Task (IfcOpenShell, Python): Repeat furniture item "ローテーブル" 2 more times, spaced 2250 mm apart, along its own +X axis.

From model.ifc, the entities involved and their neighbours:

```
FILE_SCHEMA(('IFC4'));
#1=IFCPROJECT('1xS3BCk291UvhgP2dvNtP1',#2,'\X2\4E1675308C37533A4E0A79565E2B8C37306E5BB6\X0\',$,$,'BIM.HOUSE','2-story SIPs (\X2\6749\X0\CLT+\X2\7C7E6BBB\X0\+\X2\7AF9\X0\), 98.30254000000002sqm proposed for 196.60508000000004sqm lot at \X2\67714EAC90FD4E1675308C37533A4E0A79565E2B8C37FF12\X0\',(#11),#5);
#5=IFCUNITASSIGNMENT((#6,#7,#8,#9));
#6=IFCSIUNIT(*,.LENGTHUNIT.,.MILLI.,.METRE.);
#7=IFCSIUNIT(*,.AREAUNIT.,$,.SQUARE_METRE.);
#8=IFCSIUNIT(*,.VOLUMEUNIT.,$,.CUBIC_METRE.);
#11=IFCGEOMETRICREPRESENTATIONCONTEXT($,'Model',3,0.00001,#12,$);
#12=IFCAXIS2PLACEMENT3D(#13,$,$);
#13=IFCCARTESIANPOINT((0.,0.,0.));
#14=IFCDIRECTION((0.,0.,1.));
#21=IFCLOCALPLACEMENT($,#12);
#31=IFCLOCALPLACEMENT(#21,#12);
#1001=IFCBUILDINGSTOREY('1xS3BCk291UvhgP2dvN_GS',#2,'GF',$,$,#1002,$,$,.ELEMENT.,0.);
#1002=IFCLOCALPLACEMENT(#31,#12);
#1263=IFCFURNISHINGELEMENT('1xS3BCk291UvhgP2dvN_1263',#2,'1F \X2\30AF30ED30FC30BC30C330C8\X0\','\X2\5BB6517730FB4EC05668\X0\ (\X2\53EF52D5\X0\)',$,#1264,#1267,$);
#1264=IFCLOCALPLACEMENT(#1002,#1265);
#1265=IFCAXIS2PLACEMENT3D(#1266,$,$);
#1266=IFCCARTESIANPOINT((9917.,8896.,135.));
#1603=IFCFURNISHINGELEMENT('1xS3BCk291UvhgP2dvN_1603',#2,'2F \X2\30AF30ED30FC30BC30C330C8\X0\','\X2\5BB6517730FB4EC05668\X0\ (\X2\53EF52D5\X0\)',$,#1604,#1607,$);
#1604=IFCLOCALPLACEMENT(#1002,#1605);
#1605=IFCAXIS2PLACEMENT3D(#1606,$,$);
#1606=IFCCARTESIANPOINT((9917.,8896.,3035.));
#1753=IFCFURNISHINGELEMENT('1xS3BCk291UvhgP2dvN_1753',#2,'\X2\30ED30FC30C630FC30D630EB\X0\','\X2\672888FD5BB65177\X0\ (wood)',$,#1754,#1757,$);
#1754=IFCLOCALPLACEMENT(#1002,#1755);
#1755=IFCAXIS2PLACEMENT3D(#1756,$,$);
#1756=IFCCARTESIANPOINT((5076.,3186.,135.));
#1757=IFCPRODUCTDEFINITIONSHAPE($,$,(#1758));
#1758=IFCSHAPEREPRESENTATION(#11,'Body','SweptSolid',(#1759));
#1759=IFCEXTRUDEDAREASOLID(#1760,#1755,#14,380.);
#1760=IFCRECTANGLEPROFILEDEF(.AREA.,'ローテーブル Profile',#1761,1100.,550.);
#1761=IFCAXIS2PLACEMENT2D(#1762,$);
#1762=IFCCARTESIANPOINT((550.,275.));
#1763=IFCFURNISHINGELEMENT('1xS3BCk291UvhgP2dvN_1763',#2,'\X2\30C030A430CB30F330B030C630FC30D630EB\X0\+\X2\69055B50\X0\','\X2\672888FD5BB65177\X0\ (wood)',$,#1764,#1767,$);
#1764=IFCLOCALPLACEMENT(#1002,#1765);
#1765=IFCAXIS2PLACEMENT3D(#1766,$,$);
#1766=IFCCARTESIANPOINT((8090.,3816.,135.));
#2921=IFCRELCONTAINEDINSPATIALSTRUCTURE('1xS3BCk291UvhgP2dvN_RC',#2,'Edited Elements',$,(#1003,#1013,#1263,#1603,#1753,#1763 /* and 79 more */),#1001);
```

```python
import ifcopenshell
import ifcopenshell.api.geometry
import ifcopenshell.api.root
import ifcopenshell.util.element
import ifcopenshell.util.placement
import ifcopenshell.util.unit

model = ifcopenshell.open("model.ifc")
unit_scale = ifcopenshell.util.unit.calculate_unit_scale(model)


def reuse_history(source, copy):
    """copy_class also copies each property set's owner history, people and application; keep the originals."""
    for rel in copy.IsDefinedBy:
        if rel.is_a("IfcRelDefinesByProperties") and (history := rel.RelatingPropertyDefinition.OwnerHistory):
            rel.RelatingPropertyDefinition.OwnerHistory = source.OwnerHistory
            ifcopenshell.util.element.remove_deep2(model, history)


source = model.by_id(1753)
base = ifcopenshell.util.placement.get_local_placement(source.ObjectPlacement)
step = base[:3, 0] * 2.25 / unit_scale

for i in range(1, 3):
    copy = ifcopenshell.api.root.copy_class(model, product=source)
    copy.Representation = ifcopenshell.util.element.copy_deep(
        model, source.Representation, exclude=["IfcGeometricRepresentationContext", "IfcRepresentationMap"]
    )
    reuse_history(source, copy)
    matrix = base.copy()
    matrix[:3, 3] += i * step
    print("added at", matrix[:3, 3].round(3) + 0.0)
    ifcopenshell.api.geometry.edit_object_placement(model, product=copy, matrix=matrix, is_si=False)

model.write("model_rev.ifc")
```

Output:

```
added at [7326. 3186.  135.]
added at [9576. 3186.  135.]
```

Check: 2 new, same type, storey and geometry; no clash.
